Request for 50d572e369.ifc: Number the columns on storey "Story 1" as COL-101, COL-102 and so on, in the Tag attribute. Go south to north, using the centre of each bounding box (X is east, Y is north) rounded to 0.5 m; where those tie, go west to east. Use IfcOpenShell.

First a look at what the model holds.

```python
import ifcopenshell
import ifcopenshell.util.element
import ifcopenshell.util.placement

model = ifcopenshell.open("50d572e369.ifc")
print(model.schema)
storey = next(s for s in model.by_type("IfcBuildingStorey") if s.Name == "Story 1")
columns = [e for e in ifcopenshell.util.element.get_decomposition(storey) if e.is_a("IfcColumn")]
for e in sorted(columns, key=lambda e: e.id()):
    origin = ifcopenshell.util.placement.get_local_placement(e.ObjectPlacement)[:3, 3]
    print(e.id(), e.Tag, e.Name, origin.round(2) + 0.0, sep=" | ")
```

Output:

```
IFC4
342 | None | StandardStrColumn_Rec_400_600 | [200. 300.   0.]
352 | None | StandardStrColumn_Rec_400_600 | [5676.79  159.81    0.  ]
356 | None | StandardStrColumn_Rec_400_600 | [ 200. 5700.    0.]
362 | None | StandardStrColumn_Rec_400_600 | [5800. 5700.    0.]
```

```python
import ifcopenshell
import ifcopenshell.geom
import ifcopenshell.util.element
import ifcopenshell.util.shape

model = ifcopenshell.open("50d572e369.ifc")
settings = ifcopenshell.geom.settings()
settings.set("use-world-coords", True)


def centre(element):
    shape = ifcopenshell.geom.create_shape(settings, element)
    return ifcopenshell.util.shape.get_bbox_centroid(shape.geometry)


storey = next(s for s in model.by_type("IfcBuildingStorey") if s.Name == "Story 1")
columns = [e for e in ifcopenshell.util.element.get_decomposition(storey) if e.is_a("IfcColumn")]

# Insertion points can sit at a corner or the storey origin, so sort by the geometry (in metres).
centres = {e: centre(e) for e in columns}
columns.sort(key=lambda e: (round(centres[e][1] / 0.5), centres[e][0]))

for i, e in enumerate(columns, start=1):
    number = f"COL-1{i:02d}"
    e.Tag = number
    print(e.id(), number)

model.write("50d572e369_updated.ifc")
```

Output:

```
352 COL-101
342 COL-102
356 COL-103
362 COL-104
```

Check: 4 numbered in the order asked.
